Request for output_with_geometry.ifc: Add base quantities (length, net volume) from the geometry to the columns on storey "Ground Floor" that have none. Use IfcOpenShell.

First a look at what the model holds.

```python
import ifcopenshell
import ifcopenshell.util.element
import ifcopenshell.util.unit

model = ifcopenshell.open("output_with_geometry.ifc")
print(model.schema)
for unit_type in ("LENGTHUNIT", "AREAUNIT", "VOLUMEUNIT"):
    print(unit_type, ifcopenshell.util.unit.calculate_unit_scale(model, unit_type))
storey = next(s for s in model.by_type("IfcBuildingStorey") if s.Name == "Ground Floor")
columns = [e for e in ifcopenshell.util.element.get_decomposition(storey) if e.is_a("IfcColumn")]
for e in sorted(columns, key=lambda e: e.id()):
    print(e.id(), e.is_a(), e.Name, list(ifcopenshell.util.element.get_psets(e, qtos_only=True)), sep=" | ")
```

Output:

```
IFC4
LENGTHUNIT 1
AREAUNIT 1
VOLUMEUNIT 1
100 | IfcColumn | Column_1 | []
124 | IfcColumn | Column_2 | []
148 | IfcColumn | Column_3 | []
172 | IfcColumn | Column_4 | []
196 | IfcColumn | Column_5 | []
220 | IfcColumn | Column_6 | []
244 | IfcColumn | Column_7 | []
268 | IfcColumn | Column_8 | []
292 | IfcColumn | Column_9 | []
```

```python
import ifcopenshell
import ifcopenshell.api.pset
import ifcopenshell.geom
import ifcopenshell.util.element
import ifcopenshell.util.shape
import ifcopenshell.util.unit

model = ifcopenshell.open("output_with_geometry.ifc")
unit_scale = ifcopenshell.util.unit.calculate_unit_scale(model)
volume_scale = ifcopenshell.util.unit.calculate_unit_scale(model, "VOLUMEUNIT")
settings = ifcopenshell.geom.settings()

storey = next(s for s in model.by_type("IfcBuildingStorey") if s.Name == "Ground Floor")
columns = [e for e in ifcopenshell.util.element.get_decomposition(storey) if e.is_a("IfcColumn")]

for e in sorted(columns, key=lambda e: e.id()):
    if ifcopenshell.util.element.get_psets(e, qtos_only=True, should_inherit=False):
        continue
    # Geometry comes back in metres, in the element's own axes.
    shape = ifcopenshell.geom.create_shape(settings, e)
    values = {
        "Length": ifcopenshell.util.shape.get_z(shape.geometry) / unit_scale,
        "NetVolume": ifcopenshell.util.shape.get_volume(shape.geometry) / volume_scale,
    }
    qto = ifcopenshell.api.pset.add_qto(model, product=e, name="Qto_ColumnBaseQuantities")
    ifcopenshell.api.pset.edit_qto(model, qto=qto, properties=values)
    print(e.id(), {k: round(v, 3) for k, v in values.items()})

model.write("output_with_geometry_rev.ifc")
```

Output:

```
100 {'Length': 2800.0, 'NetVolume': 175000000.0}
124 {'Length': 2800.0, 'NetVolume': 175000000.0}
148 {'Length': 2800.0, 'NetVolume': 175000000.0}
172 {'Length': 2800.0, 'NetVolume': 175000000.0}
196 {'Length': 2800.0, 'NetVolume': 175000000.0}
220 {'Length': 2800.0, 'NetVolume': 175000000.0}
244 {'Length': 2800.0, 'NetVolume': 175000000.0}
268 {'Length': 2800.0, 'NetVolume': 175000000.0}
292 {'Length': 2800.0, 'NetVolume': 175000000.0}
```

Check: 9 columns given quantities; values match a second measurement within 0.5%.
